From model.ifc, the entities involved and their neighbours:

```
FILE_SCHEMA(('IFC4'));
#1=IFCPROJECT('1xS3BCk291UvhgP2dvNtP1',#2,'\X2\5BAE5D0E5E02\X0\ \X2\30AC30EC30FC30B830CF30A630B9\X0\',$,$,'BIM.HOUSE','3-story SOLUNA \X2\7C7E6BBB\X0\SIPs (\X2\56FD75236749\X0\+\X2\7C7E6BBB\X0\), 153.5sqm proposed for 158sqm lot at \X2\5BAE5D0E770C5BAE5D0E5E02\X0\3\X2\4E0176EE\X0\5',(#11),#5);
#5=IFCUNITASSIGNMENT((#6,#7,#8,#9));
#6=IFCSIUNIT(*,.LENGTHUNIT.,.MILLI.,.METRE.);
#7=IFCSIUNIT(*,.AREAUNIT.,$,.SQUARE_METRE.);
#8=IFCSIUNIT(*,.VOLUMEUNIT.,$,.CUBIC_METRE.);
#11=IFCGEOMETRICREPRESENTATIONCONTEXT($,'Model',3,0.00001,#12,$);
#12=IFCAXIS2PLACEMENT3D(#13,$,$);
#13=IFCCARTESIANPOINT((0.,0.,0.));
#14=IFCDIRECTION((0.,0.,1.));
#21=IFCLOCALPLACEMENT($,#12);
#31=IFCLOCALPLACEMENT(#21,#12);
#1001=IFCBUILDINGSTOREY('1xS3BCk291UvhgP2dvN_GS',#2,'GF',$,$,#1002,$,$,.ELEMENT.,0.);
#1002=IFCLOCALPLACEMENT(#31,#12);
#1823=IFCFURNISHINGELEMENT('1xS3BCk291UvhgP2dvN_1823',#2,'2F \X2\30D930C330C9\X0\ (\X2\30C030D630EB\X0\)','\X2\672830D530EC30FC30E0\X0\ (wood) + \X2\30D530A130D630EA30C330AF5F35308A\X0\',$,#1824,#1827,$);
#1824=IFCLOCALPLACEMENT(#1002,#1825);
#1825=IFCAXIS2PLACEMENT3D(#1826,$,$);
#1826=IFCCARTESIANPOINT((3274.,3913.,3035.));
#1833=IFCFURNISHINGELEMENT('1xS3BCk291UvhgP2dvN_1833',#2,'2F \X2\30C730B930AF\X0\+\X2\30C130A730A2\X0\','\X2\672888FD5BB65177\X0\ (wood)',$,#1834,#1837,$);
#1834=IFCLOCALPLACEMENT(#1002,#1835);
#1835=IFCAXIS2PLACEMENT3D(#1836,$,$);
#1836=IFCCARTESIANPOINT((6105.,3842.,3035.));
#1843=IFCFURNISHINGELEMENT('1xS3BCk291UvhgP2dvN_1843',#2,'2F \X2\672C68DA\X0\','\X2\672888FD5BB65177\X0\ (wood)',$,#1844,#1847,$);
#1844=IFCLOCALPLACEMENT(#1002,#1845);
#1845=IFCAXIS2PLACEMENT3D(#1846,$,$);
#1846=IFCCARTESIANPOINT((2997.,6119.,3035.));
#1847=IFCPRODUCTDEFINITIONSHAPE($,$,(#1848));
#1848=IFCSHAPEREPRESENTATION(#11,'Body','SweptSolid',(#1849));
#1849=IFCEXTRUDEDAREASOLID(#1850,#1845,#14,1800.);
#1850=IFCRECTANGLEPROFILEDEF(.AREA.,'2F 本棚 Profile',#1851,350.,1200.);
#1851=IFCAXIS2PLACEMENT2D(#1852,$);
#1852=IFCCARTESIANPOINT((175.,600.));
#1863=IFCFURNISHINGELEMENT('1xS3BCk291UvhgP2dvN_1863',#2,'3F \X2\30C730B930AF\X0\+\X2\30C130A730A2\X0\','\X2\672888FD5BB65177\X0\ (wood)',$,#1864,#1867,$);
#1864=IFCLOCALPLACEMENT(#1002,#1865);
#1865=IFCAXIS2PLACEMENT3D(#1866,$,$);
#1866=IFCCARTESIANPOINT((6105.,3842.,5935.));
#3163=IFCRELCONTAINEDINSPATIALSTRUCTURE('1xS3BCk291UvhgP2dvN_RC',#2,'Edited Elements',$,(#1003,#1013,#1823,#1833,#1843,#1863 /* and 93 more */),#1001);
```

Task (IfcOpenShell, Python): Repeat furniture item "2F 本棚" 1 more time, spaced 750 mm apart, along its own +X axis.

```python
import ifcopenshell
import ifcopenshell.api.geometry
import ifcopenshell.api.root
import ifcopenshell.util.element
import ifcopenshell.util.placement

model = ifcopenshell.open("model.ifc")


def reuse_history(source, copy):
    """copy_class also copies each property set's owner history, people and application; keep the originals."""
    for rel in copy.IsDefinedBy:
        if rel.is_a("IfcRelDefinesByProperties") and (history := rel.RelatingPropertyDefinition.OwnerHistory):
            rel.RelatingPropertyDefinition.OwnerHistory = source.OwnerHistory
            ifcopenshell.util.element.remove_deep2(model, history)


source = model.by_id(1843)
base = ifcopenshell.util.placement.get_local_placement(source.ObjectPlacement)
step = base[:3, 0] * 750.0

for i in range(1, 2):
    copy = ifcopenshell.api.root.copy_class(model, product=source)
    copy.Representation = ifcopenshell.util.element.copy_deep(
        model, source.Representation, exclude=["IfcGeometricRepresentationContext", "IfcRepresentationMap"]
    )
    reuse_history(source, copy)
    matrix = base.copy()
    matrix[:3, 3] += i * step
    print("added at", matrix[:3, 3].round(3) + 0.0)
    ifcopenshell.api.geometry.edit_object_placement(model, product=copy, matrix=matrix, is_si=False)

model.write("model_v2.ifc")
```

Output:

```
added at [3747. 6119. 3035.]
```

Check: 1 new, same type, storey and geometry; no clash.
